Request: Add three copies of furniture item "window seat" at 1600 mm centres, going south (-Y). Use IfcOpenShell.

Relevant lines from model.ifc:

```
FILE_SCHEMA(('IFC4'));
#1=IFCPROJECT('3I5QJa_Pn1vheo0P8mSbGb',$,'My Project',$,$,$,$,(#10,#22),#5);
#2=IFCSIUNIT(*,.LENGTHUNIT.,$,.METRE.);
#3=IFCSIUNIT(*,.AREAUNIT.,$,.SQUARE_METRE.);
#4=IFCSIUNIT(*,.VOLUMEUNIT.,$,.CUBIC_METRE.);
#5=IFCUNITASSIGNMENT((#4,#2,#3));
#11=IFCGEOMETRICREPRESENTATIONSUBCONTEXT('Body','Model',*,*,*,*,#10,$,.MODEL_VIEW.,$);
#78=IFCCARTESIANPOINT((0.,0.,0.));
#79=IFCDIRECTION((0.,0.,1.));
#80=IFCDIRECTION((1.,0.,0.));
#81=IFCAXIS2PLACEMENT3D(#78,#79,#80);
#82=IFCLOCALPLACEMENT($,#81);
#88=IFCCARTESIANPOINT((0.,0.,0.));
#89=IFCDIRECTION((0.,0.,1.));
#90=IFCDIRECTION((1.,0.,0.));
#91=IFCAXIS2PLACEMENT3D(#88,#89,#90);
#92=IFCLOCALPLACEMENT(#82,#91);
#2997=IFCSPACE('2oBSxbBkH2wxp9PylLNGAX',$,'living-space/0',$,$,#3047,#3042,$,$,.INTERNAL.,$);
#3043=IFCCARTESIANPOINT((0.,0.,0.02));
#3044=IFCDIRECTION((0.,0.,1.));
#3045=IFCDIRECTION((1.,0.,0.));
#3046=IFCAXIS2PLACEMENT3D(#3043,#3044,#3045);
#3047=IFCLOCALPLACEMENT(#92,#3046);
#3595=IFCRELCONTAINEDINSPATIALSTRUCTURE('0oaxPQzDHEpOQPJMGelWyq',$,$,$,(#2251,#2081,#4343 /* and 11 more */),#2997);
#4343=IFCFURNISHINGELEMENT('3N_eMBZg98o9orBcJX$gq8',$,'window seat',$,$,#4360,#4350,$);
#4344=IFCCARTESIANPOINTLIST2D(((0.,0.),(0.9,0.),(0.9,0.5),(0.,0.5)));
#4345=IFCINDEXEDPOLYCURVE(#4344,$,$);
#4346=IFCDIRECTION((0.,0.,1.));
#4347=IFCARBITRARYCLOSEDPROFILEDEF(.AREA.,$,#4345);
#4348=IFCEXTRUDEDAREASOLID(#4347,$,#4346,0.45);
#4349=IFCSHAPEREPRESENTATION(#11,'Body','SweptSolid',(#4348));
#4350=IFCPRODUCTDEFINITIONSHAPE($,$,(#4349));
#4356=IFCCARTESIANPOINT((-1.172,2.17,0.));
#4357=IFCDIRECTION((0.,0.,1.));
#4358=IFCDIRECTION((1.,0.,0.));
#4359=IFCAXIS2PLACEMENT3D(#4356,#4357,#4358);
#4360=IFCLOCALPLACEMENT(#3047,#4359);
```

```python
import numpy as np
import ifcopenshell
import ifcopenshell.api.geometry
import ifcopenshell.api.root
import ifcopenshell.util.element
import ifcopenshell.util.placement

model = ifcopenshell.open("model.ifc")

source = model.by_guid("3N_eMBZg98o9orBcJX$gq8")
base = ifcopenshell.util.placement.get_local_placement(source.ObjectPlacement)
step = np.array([0.0, -1.0, 0.0]) * 1.6

for i in range(1, 4):
    copy = ifcopenshell.api.root.copy_class(model, product=source)
    copy.Representation = ifcopenshell.util.element.copy_deep(
        model, source.Representation, exclude=["IfcGeometricRepresentationContext", "IfcRepresentationMap"]
    )
    matrix = base.copy()
    matrix[:3, 3] += i * step
    print("added at", matrix[:3, 3].round(3) + 0.0)
    ifcopenshell.api.geometry.edit_object_placement(model, product=copy, matrix=matrix, is_si=False)

model.write("model_rev.ifc")
```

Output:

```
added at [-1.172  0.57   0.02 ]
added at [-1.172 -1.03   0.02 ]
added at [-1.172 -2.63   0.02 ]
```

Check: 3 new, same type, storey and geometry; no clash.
